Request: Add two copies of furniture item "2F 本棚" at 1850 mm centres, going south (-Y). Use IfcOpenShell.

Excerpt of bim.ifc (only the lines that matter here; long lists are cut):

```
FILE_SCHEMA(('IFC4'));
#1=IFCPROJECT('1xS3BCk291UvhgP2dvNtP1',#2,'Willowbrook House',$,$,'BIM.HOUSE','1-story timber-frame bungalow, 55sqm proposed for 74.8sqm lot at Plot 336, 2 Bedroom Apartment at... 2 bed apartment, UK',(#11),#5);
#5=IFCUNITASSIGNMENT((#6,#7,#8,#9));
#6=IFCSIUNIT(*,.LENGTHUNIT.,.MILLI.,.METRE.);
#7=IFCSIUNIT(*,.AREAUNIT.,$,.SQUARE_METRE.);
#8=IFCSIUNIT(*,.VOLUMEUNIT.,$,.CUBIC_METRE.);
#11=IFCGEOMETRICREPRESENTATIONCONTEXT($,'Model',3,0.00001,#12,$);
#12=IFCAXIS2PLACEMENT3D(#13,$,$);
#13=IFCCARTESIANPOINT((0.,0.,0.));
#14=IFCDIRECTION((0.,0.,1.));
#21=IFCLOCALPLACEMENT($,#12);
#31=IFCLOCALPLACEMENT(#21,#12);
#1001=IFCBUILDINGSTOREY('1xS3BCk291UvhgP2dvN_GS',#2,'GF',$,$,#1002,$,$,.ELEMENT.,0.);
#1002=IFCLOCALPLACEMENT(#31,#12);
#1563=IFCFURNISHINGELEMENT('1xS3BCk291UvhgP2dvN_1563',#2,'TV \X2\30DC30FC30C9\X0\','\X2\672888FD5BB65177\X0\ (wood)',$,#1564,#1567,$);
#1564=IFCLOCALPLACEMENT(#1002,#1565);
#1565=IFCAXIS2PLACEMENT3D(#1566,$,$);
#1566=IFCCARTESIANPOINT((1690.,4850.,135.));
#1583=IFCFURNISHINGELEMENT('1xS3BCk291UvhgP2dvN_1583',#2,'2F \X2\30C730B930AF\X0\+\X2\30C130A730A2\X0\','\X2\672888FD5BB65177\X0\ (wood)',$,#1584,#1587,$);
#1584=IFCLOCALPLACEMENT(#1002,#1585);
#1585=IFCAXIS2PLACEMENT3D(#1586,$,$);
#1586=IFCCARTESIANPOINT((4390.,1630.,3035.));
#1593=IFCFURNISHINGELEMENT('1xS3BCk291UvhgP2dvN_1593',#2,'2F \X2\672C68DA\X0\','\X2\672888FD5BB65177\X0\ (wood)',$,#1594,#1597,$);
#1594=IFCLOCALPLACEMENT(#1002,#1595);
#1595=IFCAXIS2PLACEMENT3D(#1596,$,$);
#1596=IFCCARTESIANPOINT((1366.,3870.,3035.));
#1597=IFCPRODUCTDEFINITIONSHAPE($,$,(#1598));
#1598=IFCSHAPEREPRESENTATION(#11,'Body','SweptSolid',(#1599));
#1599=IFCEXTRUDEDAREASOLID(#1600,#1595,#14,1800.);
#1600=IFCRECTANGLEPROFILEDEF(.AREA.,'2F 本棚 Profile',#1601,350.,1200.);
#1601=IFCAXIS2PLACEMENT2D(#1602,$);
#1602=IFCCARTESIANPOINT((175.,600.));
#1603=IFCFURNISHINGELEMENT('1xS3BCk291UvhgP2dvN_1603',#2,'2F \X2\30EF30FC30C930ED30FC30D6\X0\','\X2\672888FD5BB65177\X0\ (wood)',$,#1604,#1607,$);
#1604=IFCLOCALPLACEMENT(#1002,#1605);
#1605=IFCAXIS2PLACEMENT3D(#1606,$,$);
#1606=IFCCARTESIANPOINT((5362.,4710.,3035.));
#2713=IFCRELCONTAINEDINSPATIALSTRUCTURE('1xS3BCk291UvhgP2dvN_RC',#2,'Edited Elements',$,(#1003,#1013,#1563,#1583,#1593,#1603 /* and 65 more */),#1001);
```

```python
import numpy as np
import ifcopenshell
import ifcopenshell.api.geometry
import ifcopenshell.api.root
import ifcopenshell.util.element
import ifcopenshell.util.placement
import ifcopenshell.util.unit

model = ifcopenshell.open("bim.ifc")
unit_scale = ifcopenshell.util.unit.calculate_unit_scale(model)


def reuse_history(source, copy):
    """copy_class also copies each property set's owner history, people and application; keep the originals."""
    for rel in copy.IsDefinedBy:
        if rel.is_a("IfcRelDefinesByProperties") and (history := rel.RelatingPropertyDefinition.OwnerHistory):
            rel.RelatingPropertyDefinition.OwnerHistory = source.OwnerHistory
            ifcopenshell.util.element.remove_deep2(model, history)


source = model.by_id(1593)
base = ifcopenshell.util.placement.get_local_placement(source.ObjectPlacement)
step = np.array([0.0, -1.0, 0.0]) * 1.85 / unit_scale

for i in range(1, 3):
    copy = ifcopenshell.api.root.copy_class(model, product=source)
    copy.Representation = ifcopenshell.util.element.copy_deep(
        model, source.Representation, exclude=["IfcGeometricRepresentationContext", "IfcRepresentationMap"]
    )
    reuse_history(source, copy)
    matrix = base.copy()
    matrix[:3, 3] += i * step
    print("added at", matrix[:3, 3].round(3) + 0.0)
    ifcopenshell.api.geometry.edit_object_placement(model, product=copy, matrix=matrix, is_si=False)

model.write("bim_updated.ifc")
```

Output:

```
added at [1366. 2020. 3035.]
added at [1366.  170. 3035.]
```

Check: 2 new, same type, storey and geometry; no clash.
